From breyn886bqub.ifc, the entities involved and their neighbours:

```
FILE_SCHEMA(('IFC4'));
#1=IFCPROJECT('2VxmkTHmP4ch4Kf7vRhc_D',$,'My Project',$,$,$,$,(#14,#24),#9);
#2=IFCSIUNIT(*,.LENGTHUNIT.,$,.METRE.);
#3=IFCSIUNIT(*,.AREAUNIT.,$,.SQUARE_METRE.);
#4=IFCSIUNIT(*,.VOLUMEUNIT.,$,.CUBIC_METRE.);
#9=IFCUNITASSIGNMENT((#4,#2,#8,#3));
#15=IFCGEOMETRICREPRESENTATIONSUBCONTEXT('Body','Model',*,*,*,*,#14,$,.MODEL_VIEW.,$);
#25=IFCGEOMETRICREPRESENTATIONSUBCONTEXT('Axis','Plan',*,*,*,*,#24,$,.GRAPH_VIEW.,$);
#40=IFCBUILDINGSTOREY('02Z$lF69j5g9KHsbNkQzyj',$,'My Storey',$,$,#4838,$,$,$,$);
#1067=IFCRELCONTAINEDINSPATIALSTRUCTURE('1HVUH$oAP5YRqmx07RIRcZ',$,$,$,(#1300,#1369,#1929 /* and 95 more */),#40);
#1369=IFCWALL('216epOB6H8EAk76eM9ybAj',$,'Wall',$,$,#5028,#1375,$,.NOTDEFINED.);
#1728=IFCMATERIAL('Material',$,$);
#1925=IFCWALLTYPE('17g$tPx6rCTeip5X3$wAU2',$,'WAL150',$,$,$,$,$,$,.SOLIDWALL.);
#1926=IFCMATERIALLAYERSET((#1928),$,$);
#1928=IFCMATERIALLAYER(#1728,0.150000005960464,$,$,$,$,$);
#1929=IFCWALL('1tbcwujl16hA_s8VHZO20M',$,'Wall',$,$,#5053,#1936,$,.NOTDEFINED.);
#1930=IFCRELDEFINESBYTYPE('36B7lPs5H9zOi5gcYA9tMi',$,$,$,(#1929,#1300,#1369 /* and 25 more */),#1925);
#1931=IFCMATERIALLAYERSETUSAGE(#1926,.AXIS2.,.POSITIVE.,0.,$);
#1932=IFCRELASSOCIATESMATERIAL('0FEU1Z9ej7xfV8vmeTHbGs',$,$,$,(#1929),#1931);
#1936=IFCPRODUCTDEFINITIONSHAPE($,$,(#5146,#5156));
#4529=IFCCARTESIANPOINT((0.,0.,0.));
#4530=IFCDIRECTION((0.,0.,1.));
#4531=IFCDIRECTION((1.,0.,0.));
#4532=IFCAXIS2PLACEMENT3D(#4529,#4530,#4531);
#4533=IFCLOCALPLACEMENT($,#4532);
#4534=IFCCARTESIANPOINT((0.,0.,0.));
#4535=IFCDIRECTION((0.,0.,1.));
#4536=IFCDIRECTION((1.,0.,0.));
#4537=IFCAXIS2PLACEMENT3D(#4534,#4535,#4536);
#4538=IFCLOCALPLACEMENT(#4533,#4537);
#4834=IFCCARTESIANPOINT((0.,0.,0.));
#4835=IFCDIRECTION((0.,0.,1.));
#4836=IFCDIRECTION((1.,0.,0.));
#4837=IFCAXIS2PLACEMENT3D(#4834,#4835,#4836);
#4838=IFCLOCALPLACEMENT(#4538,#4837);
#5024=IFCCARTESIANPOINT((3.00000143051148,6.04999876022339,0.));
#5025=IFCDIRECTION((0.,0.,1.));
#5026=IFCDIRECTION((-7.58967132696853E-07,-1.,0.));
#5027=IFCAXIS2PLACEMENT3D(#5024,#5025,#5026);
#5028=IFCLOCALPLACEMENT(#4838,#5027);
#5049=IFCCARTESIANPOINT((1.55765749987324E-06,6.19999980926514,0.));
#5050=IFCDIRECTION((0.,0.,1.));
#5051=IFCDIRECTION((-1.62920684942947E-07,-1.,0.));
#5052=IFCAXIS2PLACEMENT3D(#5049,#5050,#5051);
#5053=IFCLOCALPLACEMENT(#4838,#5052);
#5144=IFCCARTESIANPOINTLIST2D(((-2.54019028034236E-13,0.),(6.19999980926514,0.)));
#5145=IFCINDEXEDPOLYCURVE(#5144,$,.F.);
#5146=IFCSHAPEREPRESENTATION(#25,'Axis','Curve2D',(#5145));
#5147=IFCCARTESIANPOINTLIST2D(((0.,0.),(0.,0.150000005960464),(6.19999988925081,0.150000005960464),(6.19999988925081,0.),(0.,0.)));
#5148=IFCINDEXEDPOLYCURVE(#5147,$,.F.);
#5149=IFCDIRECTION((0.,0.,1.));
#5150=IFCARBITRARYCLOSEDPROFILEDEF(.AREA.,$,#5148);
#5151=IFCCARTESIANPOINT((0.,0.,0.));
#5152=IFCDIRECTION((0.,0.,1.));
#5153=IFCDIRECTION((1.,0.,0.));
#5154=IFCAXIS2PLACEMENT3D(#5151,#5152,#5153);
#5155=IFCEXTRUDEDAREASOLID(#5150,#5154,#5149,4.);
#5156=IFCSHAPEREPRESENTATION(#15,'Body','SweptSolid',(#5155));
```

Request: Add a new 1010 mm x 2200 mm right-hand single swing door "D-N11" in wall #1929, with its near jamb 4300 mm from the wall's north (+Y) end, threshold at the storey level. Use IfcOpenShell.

```python
import numpy as np
import ifcopenshell
import ifcopenshell.api.feature
import ifcopenshell.api.geometry
import ifcopenshell.api.root
import ifcopenshell.api.spatial
import ifcopenshell.geom
import ifcopenshell.util.element
import ifcopenshell.util.placement
import ifcopenshell.util.representation
import ifcopenshell.util.shape
import ifcopenshell.util.unit

model = ifcopenshell.open("breyn886bqub.ifc")
unit_scale = ifcopenshell.util.unit.calculate_unit_scale(model)
settings = ifcopenshell.geom.settings()


def volume(element):
    """Net volume in cubic metres, openings subtracted."""
    shape = ifcopenshell.geom.create_shape(settings, element)
    return ifcopenshell.util.shape.get_volume(shape.geometry)


wall = model.by_guid("1tbcwujl16hA_s8VHZO20M")
storey = ifcopenshell.util.element.get_container(wall, ifc_class="IfcBuildingStorey")
context = ifcopenshell.util.representation.get_context(model, "Model", "Body", "MODEL_VIEW")
before = volume(wall)

width, height, from_end, sill = 1.01, 2.2, 4.3, 0.0  # metres

# The wall runs along its own X axis, and the end named is its -X end.
wall_shape = ifcopenshell.geom.create_shape(settings, wall)
x, y, z = ifcopenshell.util.shape.get_vertices(wall_shape.geometry).T
start = x.min() + from_end
face, thickness = float(y.min()), float(y.max() - y.min())
wall_matrix = ifcopenshell.util.placement.get_local_placement(wall.ObjectPlacement)
level = ifcopenshell.util.placement.get_local_placement(storey.ObjectPlacement)[2, 3]


def in_wall(x, y):
    """Placement at x, y metres in the wall's axes, at sill height."""
    matrix = wall_matrix.copy()
    matrix[:, 3] = wall_matrix @ np.array([x / unit_scale, y / unit_scale, 0.0, 1.0])
    matrix[2, 3] = level + sill / unit_scale
    return matrix


# Opening: a box that overshoots both wall faces by 50 mm.
opening = ifcopenshell.api.root.create_entity(model, ifc_class="IfcOpeningElement", predefined_type="OPENING")
box = ifcopenshell.api.geometry.add_wall_representation(
    model, context=context, length=width, height=height, thickness=thickness + 0.1
)
ifcopenshell.api.geometry.assign_representation(model, product=opening, representation=box)
ifcopenshell.api.geometry.edit_object_placement(model, product=opening, matrix=in_wall(start, face - 0.05), is_si=False)
ifcopenshell.api.feature.add_feature(model, feature=opening, element=wall)

door = ifcopenshell.api.root.create_entity(model, ifc_class="IfcDoor", name="D-N11", predefined_type="DOOR")
door.OverallWidth, door.OverallHeight = width / unit_scale, height / unit_scale
door.OperationType = "SINGLE_SWING_RIGHT"
body = ifcopenshell.api.geometry.add_door_representation(
    model,
    context=context,
    overall_width=door.OverallWidth,
    overall_height=door.OverallHeight,
    operation_type="SINGLE_SWING_RIGHT",
    lining_properties={"LiningDepth": thickness / unit_scale, "ThresholdDepth": thickness / unit_scale},
)
ifcopenshell.api.geometry.assign_representation(model, product=door, representation=body)
ifcopenshell.api.spatial.assign_container(model, products=[door], relating_structure=storey)
ifcopenshell.api.feature.add_filling(model, opening=opening, element=door)

# The lining spans the wall, so the door starts at the wall face.
ifcopenshell.api.geometry.edit_object_placement(model, product=door, matrix=in_wall(start, face), is_si=False)

after = volume(wall)

print(f"wall volume {before:.3f} -> {after:.3f} m3")

model.write("breyn886bqub_edited.ifc")
```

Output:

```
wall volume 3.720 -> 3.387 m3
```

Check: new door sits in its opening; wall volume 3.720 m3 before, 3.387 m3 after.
